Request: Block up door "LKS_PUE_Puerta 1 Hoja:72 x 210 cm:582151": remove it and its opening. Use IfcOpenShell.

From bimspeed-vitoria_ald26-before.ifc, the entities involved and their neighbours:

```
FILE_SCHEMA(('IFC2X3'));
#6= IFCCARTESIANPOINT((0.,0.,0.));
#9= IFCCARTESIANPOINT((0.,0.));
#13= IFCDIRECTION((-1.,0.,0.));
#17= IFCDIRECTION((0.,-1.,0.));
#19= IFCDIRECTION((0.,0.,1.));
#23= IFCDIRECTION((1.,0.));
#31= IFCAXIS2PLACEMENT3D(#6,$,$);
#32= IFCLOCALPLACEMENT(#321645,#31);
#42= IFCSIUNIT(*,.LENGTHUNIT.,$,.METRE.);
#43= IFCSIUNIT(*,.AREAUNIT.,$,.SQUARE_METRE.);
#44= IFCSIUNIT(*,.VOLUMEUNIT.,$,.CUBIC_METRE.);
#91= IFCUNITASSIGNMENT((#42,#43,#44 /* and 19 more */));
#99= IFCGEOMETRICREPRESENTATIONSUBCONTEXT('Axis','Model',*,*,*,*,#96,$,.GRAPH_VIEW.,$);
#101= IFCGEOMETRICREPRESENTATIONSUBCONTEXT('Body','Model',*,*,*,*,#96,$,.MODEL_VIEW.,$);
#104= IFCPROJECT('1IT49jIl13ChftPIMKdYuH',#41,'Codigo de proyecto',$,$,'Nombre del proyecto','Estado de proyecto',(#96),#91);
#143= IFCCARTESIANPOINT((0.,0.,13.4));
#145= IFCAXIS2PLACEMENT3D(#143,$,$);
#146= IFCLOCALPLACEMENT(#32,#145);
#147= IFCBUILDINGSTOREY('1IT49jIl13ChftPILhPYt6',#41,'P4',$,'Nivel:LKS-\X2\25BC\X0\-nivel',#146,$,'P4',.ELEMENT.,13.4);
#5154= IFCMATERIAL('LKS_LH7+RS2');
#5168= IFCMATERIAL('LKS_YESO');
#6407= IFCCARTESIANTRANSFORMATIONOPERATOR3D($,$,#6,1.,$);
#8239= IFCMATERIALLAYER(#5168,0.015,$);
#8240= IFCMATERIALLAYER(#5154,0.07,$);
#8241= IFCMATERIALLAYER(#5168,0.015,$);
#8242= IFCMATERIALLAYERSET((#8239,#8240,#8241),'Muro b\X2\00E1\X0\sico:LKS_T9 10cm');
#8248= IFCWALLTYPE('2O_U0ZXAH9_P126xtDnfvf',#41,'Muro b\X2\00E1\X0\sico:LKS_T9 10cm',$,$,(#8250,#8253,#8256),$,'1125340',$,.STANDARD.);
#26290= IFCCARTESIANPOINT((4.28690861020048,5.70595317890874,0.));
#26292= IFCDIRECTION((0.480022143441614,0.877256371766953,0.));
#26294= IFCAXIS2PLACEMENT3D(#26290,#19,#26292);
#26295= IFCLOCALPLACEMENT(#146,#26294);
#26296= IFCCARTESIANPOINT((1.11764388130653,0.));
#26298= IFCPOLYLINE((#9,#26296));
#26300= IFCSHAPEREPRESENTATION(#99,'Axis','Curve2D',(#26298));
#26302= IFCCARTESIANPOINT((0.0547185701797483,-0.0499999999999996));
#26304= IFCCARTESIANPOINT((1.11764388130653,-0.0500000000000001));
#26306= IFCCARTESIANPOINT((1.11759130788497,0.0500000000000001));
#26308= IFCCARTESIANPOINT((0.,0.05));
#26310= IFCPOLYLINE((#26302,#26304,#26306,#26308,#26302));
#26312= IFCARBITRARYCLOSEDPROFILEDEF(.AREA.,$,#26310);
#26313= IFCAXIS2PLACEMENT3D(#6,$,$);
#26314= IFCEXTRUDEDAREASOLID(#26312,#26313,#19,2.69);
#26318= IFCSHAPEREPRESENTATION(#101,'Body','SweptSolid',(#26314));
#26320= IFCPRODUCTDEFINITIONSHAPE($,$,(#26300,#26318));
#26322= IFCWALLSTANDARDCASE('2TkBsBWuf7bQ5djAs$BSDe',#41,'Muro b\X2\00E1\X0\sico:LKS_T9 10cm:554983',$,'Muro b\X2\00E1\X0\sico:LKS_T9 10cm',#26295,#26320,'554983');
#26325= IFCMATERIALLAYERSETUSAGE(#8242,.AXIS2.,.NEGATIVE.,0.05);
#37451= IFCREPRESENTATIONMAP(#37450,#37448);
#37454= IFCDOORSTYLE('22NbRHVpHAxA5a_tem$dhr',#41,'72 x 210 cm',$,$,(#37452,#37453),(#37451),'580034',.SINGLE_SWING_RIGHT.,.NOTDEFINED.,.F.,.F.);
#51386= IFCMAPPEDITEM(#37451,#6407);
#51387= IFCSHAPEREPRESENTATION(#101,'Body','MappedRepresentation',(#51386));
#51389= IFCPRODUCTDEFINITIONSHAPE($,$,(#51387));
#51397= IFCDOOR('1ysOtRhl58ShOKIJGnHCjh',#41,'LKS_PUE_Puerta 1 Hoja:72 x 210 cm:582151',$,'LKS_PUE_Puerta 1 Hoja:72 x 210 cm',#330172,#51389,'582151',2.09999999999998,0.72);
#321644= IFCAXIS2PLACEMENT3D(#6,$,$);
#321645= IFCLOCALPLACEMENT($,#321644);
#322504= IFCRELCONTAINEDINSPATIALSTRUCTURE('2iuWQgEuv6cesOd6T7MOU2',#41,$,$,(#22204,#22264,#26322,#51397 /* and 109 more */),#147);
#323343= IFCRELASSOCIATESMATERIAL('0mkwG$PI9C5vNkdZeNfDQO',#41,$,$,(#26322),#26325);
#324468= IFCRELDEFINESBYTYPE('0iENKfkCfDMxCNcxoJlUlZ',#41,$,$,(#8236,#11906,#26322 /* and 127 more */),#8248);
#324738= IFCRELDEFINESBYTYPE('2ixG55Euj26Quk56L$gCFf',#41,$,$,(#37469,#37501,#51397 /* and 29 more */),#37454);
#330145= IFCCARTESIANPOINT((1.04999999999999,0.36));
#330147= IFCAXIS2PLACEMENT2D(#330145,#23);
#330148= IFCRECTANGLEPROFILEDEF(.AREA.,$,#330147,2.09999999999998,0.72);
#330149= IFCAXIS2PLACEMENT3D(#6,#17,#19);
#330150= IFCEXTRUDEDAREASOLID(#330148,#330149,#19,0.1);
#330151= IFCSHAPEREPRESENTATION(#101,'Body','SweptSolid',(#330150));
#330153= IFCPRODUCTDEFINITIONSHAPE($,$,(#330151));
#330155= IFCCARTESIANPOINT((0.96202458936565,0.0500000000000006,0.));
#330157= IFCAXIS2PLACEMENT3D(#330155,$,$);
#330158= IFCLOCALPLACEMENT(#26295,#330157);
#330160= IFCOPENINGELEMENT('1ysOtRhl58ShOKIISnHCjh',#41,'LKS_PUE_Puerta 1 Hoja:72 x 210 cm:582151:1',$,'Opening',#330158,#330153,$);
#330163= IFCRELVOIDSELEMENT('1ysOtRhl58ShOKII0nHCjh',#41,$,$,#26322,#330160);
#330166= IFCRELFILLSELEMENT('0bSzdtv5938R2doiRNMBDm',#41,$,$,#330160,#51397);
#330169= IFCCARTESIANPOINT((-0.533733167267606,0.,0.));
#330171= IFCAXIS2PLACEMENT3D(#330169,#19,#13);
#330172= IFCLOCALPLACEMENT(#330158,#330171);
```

```python
import ifcopenshell
import ifcopenshell.api.feature
import ifcopenshell.api.root
import ifcopenshell.geom
import ifcopenshell.util.shape

model = ifcopenshell.open("bimspeed-vitoria_ald26-before.ifc")
settings = ifcopenshell.geom.settings()


def volume(element):
    """Net volume in cubic metres, openings subtracted."""
    shape = ifcopenshell.geom.create_shape(settings, element)
    return ifcopenshell.util.shape.get_volume(shape.geometry)


door = model.by_guid("1ysOtRhl58ShOKIJGnHCjh")
opening = door.FillsVoids[0].RelatingOpeningElement
wall = opening.VoidsElements[0].RelatingBuildingElement
before = volume(wall)

ifcopenshell.api.root.remove_product(model, product=door)
ifcopenshell.api.feature.remove_feature(model, feature=opening)

after = volume(wall)

print(f"wall volume {before:.3f} -> {after:.3f} m3")

model.write("bimspeed-vitoria_ald26-before_v2.ifc")
```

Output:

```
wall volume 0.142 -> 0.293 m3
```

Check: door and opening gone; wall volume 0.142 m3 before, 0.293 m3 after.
